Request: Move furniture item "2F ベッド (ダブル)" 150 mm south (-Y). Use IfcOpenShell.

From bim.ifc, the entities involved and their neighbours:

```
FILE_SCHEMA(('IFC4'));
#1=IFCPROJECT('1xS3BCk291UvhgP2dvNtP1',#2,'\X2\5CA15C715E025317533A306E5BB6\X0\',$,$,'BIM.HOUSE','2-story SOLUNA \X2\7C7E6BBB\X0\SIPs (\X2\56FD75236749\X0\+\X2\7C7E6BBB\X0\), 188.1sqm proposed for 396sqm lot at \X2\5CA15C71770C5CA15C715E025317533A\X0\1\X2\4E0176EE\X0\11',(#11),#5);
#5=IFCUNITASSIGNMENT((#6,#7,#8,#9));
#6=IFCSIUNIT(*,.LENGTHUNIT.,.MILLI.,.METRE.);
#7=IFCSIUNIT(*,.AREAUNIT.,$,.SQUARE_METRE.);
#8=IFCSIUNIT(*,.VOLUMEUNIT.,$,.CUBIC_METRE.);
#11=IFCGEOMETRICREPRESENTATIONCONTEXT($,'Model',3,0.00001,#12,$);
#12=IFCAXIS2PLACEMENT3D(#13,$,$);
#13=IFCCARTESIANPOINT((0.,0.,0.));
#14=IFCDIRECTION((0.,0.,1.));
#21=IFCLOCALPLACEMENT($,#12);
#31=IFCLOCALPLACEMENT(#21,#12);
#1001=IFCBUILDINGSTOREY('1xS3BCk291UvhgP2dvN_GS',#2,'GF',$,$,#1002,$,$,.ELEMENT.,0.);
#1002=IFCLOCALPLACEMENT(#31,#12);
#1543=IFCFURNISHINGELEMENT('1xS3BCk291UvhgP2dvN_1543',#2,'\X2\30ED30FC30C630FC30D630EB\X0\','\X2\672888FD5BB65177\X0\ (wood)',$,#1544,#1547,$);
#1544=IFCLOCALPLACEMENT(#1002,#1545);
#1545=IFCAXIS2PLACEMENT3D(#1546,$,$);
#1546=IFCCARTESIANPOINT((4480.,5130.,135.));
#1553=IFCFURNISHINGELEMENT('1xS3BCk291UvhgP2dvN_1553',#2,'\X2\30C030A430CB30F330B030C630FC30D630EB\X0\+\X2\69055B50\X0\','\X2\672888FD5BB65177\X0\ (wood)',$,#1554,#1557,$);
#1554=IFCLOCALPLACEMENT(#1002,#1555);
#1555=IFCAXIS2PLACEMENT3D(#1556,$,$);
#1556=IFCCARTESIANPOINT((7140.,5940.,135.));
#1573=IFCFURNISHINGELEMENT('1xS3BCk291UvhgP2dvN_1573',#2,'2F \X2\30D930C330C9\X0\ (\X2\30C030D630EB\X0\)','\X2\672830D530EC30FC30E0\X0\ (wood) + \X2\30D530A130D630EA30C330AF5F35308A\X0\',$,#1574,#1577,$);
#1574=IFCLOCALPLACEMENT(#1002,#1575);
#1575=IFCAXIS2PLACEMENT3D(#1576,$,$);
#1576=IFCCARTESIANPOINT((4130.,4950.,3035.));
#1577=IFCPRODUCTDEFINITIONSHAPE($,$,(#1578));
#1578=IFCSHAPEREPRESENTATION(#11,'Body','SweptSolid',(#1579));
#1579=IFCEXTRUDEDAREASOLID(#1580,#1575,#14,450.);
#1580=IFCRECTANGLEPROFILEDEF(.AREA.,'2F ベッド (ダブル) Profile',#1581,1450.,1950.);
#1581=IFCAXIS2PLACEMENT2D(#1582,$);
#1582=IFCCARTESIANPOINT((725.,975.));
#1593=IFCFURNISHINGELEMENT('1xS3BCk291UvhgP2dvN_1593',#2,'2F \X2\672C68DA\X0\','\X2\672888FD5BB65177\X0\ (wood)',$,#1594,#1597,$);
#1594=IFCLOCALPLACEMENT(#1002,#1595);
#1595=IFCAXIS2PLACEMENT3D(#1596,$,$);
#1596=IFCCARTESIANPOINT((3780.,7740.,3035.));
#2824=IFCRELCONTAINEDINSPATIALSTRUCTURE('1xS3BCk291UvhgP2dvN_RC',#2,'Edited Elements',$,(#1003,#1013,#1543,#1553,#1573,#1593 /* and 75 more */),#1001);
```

```python
import ifcopenshell
import ifcopenshell.api.geometry
import ifcopenshell.util.placement
import ifcopenshell.util.unit

model = ifcopenshell.open("bim.ifc")
unit_scale = ifcopenshell.util.unit.calculate_unit_scale(model)

item = model.by_guid("1xS3BCk291UvhgP2dvN_1573")
matrix = ifcopenshell.util.placement.get_local_placement(item.ObjectPlacement)
matrix[1, 3] -= 0.15 / unit_scale
ifcopenshell.api.geometry.edit_object_placement(model, product=item, matrix=matrix, is_si=False)

print(ifcopenshell.util.placement.get_local_placement(item.ObjectPlacement).round(3) + 0.0)

model.write("bim_edited.ifc")
```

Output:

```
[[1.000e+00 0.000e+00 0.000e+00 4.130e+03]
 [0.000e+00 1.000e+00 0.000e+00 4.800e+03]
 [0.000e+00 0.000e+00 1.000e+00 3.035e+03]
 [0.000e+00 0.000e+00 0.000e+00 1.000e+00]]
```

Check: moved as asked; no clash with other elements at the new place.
